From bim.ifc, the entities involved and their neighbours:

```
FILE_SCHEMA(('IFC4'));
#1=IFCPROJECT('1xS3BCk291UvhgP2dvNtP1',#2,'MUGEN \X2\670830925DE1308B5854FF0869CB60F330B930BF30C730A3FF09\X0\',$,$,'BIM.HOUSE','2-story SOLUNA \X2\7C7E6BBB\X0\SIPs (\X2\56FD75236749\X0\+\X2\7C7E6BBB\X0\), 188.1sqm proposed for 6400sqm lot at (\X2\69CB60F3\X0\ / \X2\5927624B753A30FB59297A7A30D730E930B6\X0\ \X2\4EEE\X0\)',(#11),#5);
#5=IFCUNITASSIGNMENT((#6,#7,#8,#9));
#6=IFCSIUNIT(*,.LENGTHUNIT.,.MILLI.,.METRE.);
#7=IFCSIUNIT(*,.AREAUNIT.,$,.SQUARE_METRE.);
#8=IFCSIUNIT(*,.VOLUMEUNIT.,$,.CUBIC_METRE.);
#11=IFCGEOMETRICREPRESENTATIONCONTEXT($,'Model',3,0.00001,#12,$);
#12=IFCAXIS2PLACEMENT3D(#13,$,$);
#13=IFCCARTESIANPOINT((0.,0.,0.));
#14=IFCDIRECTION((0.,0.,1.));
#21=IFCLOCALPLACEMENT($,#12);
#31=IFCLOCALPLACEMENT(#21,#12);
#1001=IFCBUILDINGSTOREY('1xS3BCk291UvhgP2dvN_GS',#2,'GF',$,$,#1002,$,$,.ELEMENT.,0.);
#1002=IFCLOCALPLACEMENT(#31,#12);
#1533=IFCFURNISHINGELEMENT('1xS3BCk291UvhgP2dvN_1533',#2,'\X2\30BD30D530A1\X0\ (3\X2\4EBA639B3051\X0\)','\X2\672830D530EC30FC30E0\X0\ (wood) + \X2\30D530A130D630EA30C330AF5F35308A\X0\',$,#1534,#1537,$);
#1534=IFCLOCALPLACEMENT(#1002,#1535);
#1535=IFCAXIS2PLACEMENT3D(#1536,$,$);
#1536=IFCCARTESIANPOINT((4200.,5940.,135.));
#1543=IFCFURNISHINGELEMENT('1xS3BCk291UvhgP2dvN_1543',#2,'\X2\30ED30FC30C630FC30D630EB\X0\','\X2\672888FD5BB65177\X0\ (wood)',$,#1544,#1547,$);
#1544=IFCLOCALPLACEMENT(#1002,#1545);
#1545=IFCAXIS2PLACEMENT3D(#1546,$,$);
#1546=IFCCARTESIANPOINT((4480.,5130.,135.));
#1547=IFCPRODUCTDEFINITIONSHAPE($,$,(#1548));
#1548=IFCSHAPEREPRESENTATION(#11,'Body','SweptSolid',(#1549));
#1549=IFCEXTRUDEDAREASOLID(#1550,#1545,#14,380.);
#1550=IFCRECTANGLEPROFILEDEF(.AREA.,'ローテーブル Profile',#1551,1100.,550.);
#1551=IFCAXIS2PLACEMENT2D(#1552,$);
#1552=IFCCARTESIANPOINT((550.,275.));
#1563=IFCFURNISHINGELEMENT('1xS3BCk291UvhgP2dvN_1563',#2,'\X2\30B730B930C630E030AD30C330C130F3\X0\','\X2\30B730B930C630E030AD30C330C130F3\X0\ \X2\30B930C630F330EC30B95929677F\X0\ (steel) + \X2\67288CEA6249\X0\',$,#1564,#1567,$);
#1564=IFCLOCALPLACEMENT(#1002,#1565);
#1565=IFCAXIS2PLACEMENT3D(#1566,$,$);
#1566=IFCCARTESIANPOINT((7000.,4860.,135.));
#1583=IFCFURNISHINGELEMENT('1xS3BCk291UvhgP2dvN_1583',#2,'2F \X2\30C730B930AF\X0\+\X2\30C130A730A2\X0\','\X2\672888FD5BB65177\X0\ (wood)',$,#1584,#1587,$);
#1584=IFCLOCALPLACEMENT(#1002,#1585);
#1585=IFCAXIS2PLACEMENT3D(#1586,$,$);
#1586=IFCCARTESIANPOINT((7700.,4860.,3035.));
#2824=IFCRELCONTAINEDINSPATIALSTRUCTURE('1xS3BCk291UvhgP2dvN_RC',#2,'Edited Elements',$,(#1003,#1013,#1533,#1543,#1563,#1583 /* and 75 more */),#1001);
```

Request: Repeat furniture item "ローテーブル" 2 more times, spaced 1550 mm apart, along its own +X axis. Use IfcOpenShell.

```python
import ifcopenshell
import ifcopenshell.api.geometry
import ifcopenshell.api.root
import ifcopenshell.util.element
import ifcopenshell.util.placement

model = ifcopenshell.open("bim.ifc")


def reuse_history(source, copy):
    """copy_class also copies each property set's owner history, people and application; keep the originals."""
    for rel in copy.IsDefinedBy:
        if rel.is_a("IfcRelDefinesByProperties") and (history := rel.RelatingPropertyDefinition.OwnerHistory):
            rel.RelatingPropertyDefinition.OwnerHistory = source.OwnerHistory
            ifcopenshell.util.element.remove_deep2(model, history)


source = model.by_guid("1xS3BCk291UvhgP2dvN_1543")
base = ifcopenshell.util.placement.get_local_placement(source.ObjectPlacement)
step = base[:3, 0] * 1550.0

for i in range(1, 3):
    copy = ifcopenshell.api.root.copy_class(model, product=source)
    copy.Representation = ifcopenshell.util.element.copy_deep(
        model, source.Representation, exclude=["IfcGeometricRepresentationContext", "IfcRepresentationMap"]
    )
    reuse_history(source, copy)
    matrix = base.copy()
    matrix[:3, 3] += i * step
    print("added at", matrix[:3, 3].round(3) + 0.0)
    ifcopenshell.api.geometry.edit_object_placement(model, product=copy, matrix=matrix, is_si=False)

model.write("bim_edited.ifc")
```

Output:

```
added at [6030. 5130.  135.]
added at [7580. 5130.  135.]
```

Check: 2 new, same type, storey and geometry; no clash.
